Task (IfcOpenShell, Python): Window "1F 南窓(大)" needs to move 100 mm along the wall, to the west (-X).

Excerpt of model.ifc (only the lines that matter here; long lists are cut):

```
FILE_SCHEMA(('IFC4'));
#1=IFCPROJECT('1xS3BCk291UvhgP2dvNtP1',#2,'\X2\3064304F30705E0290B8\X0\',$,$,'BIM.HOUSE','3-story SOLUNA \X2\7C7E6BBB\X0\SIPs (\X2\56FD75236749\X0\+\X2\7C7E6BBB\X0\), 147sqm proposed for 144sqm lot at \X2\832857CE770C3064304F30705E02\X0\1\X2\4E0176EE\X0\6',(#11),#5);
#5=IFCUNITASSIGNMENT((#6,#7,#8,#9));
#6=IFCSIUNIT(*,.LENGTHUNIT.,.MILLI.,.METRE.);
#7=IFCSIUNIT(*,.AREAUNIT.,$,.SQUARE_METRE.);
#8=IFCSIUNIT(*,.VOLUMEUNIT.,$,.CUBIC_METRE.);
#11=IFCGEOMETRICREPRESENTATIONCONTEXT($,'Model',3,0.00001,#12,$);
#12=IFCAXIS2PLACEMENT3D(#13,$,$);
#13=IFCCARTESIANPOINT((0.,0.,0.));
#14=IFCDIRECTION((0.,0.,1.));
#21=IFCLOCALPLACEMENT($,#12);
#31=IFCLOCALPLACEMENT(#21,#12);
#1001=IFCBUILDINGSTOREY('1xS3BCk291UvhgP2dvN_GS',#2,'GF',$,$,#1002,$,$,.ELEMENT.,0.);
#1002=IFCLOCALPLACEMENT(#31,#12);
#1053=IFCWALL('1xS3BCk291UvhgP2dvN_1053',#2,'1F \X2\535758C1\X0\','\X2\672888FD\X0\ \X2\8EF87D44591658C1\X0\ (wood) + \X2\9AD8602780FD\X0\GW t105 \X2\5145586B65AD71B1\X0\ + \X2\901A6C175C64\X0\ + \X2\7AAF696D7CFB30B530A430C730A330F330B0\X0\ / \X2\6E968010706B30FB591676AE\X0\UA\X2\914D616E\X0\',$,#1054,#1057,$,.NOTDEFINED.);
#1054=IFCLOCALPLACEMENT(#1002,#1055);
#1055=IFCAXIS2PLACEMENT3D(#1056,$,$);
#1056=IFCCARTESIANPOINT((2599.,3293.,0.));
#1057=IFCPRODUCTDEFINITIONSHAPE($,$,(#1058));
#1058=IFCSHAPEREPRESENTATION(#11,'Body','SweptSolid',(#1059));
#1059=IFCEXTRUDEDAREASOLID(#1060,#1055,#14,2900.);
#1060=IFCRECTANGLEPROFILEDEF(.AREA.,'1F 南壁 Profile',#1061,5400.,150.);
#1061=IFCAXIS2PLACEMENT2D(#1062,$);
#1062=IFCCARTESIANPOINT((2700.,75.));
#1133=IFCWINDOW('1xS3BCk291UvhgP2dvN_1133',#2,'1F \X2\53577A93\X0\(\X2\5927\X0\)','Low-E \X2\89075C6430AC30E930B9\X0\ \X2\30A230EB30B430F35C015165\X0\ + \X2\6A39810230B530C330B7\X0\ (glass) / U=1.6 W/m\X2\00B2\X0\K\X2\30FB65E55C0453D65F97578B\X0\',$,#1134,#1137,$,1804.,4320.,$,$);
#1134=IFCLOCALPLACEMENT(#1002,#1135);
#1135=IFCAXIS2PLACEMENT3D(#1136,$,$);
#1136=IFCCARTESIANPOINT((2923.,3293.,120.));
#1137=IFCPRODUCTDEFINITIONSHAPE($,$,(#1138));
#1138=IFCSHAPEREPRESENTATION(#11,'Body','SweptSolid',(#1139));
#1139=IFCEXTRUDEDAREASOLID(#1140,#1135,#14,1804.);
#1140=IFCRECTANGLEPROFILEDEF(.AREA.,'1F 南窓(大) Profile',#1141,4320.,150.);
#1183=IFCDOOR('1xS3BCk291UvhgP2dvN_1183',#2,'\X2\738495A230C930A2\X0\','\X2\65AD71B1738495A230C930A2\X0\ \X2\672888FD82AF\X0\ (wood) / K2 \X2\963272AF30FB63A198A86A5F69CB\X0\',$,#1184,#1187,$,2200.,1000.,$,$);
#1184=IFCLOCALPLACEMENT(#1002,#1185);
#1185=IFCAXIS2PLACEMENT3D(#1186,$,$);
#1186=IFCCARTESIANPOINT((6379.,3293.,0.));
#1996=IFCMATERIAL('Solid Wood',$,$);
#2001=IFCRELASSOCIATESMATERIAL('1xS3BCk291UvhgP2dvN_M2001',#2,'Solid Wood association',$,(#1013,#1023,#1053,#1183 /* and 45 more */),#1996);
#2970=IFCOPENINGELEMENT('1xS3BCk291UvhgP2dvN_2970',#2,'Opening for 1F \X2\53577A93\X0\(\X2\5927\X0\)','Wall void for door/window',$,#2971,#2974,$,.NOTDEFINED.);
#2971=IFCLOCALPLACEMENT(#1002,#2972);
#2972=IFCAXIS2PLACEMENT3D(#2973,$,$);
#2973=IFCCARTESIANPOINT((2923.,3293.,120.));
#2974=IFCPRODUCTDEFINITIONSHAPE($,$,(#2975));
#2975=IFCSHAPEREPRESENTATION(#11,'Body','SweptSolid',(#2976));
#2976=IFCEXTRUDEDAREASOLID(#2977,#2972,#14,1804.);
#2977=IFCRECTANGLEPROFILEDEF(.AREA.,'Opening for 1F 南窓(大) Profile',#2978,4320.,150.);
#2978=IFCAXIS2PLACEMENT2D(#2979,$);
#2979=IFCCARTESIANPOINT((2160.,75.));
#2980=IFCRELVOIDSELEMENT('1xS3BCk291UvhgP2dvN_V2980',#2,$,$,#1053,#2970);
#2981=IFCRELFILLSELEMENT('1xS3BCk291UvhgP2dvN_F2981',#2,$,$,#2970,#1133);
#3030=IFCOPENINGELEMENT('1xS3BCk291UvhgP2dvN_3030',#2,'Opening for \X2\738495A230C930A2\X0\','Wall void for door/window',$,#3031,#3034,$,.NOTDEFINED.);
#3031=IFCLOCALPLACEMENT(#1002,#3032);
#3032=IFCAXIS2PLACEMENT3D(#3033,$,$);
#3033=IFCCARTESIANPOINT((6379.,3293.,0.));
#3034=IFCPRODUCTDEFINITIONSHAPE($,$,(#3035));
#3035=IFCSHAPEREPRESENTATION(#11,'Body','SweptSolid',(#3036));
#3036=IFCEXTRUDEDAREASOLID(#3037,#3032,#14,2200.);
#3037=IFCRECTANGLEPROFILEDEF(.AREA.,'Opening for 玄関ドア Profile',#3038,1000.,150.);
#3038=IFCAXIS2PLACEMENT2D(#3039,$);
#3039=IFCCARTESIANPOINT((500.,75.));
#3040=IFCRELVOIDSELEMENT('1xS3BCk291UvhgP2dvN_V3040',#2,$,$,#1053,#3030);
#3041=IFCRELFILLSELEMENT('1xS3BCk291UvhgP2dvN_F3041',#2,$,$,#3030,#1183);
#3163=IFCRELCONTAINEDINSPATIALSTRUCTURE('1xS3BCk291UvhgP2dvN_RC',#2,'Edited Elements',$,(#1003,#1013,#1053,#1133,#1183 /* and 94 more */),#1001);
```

```python
import ifcopenshell
import ifcopenshell.api.geometry
import ifcopenshell.util.placement

model = ifcopenshell.open("model.ifc")

window = model.by_guid("1xS3BCk291UvhgP2dvN_1133")
opening = window.FillsVoids[0].RelatingOpeningElement
wall = opening.VoidsElements[0].RelatingBuildingElement

wall_matrix = ifcopenshell.util.placement.get_local_placement(wall.ObjectPlacement)
shift = wall_matrix[:3, 0] * -100.0
before = ifcopenshell.util.placement.get_local_placement(window.ObjectPlacement)[:3, 3].copy()

# The window is not placed relative to its opening, so move both.
for product in (opening, window):
    matrix = ifcopenshell.util.placement.get_local_placement(product.ObjectPlacement)
    matrix[:3, 3] += shift
    ifcopenshell.api.geometry.edit_object_placement(model, product=product, matrix=matrix, is_si=False)

after = ifcopenshell.util.placement.get_local_placement(window.ObjectPlacement)[:3, 3]
print("window moved by", (after - before).round(3) + 0.0)

model.write("model_v2.ifc")
```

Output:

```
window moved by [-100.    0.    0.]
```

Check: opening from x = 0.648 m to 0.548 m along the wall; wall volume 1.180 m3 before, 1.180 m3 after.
